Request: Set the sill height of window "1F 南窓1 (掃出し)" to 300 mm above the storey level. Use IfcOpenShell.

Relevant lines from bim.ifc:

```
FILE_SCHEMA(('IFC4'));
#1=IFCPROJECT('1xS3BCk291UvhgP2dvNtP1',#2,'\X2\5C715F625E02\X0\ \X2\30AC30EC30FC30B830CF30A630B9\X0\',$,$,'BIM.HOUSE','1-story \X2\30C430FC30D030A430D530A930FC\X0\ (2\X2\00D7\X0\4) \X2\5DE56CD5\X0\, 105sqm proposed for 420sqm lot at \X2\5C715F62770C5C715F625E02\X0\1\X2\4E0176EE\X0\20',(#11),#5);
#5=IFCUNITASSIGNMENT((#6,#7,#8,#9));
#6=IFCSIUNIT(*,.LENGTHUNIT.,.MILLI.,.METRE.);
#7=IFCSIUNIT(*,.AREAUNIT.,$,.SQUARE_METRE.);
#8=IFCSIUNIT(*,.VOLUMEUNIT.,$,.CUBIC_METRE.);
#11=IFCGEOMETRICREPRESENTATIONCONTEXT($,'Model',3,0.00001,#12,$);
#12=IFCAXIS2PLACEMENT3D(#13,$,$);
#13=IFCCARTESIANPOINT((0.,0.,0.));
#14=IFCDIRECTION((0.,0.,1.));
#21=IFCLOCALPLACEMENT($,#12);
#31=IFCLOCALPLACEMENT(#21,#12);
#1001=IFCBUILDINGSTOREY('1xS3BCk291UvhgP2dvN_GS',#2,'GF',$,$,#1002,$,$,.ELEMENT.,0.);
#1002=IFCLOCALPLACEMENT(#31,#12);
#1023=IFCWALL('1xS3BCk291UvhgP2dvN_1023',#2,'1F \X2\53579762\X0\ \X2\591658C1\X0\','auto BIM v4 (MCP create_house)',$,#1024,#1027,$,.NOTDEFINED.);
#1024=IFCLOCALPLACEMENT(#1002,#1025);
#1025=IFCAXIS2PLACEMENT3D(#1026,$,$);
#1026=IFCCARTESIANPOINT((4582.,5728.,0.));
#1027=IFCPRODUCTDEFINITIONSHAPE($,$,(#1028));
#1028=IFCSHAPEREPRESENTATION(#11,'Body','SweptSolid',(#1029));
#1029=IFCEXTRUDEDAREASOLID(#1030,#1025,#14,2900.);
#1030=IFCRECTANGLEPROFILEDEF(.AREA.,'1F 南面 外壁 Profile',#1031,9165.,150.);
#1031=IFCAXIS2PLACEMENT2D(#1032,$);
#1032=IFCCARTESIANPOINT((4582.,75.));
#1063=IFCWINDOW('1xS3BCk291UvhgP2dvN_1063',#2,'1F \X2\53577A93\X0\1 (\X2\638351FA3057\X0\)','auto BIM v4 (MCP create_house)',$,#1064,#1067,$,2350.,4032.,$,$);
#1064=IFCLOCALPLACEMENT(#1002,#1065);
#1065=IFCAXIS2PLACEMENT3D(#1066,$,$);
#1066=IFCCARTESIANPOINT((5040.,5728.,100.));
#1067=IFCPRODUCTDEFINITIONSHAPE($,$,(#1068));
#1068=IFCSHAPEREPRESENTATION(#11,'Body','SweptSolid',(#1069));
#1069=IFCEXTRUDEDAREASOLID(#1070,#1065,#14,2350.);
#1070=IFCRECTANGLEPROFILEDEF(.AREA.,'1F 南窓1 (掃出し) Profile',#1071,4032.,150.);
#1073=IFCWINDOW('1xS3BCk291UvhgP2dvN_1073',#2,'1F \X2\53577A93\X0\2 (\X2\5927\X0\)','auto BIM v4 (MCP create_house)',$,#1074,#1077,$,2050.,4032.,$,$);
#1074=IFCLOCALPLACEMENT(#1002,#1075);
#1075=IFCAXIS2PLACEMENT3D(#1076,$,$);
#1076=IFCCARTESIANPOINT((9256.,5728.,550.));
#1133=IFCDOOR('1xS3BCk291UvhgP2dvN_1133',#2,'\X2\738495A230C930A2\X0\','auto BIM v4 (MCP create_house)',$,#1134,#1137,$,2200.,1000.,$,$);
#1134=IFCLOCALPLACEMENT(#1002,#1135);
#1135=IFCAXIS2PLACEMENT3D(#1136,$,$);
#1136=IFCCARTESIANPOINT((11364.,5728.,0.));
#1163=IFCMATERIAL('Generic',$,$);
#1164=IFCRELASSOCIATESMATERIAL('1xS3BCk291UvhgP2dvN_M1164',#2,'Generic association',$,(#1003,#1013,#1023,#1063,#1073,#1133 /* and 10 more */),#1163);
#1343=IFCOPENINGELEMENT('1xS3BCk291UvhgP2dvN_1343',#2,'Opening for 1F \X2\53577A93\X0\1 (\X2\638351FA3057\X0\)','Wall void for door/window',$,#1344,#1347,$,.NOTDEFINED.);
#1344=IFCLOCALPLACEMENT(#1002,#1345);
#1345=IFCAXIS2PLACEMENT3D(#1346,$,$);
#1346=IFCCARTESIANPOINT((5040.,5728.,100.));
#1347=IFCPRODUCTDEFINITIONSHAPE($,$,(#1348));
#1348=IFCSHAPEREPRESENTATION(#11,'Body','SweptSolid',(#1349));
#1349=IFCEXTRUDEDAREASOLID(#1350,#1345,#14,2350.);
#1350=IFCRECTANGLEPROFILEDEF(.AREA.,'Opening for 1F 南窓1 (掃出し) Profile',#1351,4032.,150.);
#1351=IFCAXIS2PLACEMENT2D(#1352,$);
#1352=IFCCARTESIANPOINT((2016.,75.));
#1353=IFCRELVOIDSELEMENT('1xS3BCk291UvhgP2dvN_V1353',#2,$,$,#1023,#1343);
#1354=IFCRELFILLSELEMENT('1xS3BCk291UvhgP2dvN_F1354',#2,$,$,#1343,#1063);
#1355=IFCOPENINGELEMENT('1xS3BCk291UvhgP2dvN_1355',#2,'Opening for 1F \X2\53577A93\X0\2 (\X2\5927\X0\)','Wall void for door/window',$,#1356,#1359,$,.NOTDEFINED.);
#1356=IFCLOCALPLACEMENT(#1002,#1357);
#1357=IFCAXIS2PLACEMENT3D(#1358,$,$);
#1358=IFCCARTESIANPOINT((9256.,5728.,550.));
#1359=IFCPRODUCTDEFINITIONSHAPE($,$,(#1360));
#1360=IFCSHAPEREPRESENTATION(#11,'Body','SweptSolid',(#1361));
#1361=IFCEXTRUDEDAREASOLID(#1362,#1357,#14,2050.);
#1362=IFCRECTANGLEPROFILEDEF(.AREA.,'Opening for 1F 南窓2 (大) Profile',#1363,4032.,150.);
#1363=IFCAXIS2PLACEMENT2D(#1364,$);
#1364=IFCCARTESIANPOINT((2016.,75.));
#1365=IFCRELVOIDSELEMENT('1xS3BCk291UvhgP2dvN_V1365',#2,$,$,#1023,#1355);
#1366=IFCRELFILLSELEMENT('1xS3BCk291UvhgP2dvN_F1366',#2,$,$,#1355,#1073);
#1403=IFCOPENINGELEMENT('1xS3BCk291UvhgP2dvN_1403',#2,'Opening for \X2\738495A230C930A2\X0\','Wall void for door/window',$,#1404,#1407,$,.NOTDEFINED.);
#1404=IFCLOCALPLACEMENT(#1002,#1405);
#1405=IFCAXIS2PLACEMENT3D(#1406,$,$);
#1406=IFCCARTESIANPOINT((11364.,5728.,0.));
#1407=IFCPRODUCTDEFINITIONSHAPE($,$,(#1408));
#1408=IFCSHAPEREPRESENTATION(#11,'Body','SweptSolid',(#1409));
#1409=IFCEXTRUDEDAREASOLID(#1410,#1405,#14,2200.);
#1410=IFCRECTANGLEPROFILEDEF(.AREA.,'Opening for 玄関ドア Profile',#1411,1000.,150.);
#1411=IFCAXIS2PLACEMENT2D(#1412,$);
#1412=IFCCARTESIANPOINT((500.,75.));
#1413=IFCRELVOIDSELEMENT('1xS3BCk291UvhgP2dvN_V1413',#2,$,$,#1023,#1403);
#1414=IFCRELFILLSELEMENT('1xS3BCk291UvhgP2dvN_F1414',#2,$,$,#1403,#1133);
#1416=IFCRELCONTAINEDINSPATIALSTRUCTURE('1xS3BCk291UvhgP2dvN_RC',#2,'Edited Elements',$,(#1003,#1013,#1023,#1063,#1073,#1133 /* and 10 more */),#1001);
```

```python
import numpy as np
import ifcopenshell
import ifcopenshell.api.geometry
import ifcopenshell.geom
import ifcopenshell.util.element
import ifcopenshell.util.placement
import ifcopenshell.util.shape
import ifcopenshell.util.unit

model = ifcopenshell.open("bim.ifc")
unit_scale = ifcopenshell.util.unit.calculate_unit_scale(model)

window = model.by_guid("1xS3BCk291UvhgP2dvN_1063")
opening = window.FillsVoids[0].RelatingOpeningElement
storey = ifcopenshell.util.element.get_container(window, ifc_class="IfcBuildingStorey")
level = ifcopenshell.util.placement.get_local_placement(storey.ObjectPlacement)[2, 3]

# The opening's origin need not be at the sill, so measure its lowest point.
shape = ifcopenshell.geom.create_shape(ifcopenshell.geom.settings(), opening)
bottom = ifcopenshell.util.shape.get_shape_bottom_elevation(shape, shape.geometry) / unit_scale
dz = level + 300.0 - bottom

shift = np.array([0.0, 0.0, dz])
# The window is not placed relative to its opening, so move both.
for product in (opening, window):
    matrix = ifcopenshell.util.placement.get_local_placement(product.ObjectPlacement)
    matrix[:3, 3] += shift
    ifcopenshell.api.geometry.edit_object_placement(model, product=product, matrix=matrix, is_si=False)

print(f"moved by {dz * unit_scale:+.3f} m")

model.write("bim-out.ifc")
```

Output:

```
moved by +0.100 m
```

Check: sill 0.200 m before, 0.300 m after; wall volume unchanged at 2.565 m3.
